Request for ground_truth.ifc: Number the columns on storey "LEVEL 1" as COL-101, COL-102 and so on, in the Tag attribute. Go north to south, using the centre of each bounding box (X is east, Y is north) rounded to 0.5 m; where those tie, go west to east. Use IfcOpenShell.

First a look at what the model holds.

```python
import ifcopenshell
import ifcopenshell.util.element
import ifcopenshell.util.placement

model = ifcopenshell.open("ground_truth.ifc")
print(model.schema)
storey = next(s for s in model.by_type("IfcBuildingStorey") if s.Name == "LEVEL 1")
columns = [e for e in ifcopenshell.util.element.get_decomposition(storey) if e.is_a("IfcColumn")]
for e in sorted(columns, key=lambda e: e.id()):
    origin = ifcopenshell.util.placement.get_local_placement(e.ObjectPlacement)[:3, 3]
    print(e.id(), e.Tag, e.Name, origin.round(2) + 0.0, sep=" | ")
```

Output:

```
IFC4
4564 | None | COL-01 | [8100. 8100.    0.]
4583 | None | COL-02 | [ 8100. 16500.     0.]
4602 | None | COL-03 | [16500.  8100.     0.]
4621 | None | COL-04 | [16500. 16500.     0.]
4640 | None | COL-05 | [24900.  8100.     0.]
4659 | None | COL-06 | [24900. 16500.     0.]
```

```python
import ifcopenshell
import ifcopenshell.geom
import ifcopenshell.util.element
import ifcopenshell.util.shape

model = ifcopenshell.open("ground_truth.ifc")
settings = ifcopenshell.geom.settings()
settings.set("use-world-coords", True)


def centre(element):
    shape = ifcopenshell.geom.create_shape(settings, element)
    return ifcopenshell.util.shape.get_bbox_centroid(shape.geometry)


storey = next(s for s in model.by_type("IfcBuildingStorey") if s.Name == "LEVEL 1")
columns = [e for e in ifcopenshell.util.element.get_decomposition(storey) if e.is_a("IfcColumn")]

# Insertion points can sit at a corner or the storey origin, so sort by the geometry (in metres).
centres = {e: centre(e) for e in columns}
columns.sort(key=lambda e: (-round(centres[e][1] / 0.5), centres[e][0]))

for i, e in enumerate(columns, start=1):
    number = f"COL-1{i:02d}"
    e.Tag = number
    print(e.id(), number)

model.write("ground_truth-out.ifc")
```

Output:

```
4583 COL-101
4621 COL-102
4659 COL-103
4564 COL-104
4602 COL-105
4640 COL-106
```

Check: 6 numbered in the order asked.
